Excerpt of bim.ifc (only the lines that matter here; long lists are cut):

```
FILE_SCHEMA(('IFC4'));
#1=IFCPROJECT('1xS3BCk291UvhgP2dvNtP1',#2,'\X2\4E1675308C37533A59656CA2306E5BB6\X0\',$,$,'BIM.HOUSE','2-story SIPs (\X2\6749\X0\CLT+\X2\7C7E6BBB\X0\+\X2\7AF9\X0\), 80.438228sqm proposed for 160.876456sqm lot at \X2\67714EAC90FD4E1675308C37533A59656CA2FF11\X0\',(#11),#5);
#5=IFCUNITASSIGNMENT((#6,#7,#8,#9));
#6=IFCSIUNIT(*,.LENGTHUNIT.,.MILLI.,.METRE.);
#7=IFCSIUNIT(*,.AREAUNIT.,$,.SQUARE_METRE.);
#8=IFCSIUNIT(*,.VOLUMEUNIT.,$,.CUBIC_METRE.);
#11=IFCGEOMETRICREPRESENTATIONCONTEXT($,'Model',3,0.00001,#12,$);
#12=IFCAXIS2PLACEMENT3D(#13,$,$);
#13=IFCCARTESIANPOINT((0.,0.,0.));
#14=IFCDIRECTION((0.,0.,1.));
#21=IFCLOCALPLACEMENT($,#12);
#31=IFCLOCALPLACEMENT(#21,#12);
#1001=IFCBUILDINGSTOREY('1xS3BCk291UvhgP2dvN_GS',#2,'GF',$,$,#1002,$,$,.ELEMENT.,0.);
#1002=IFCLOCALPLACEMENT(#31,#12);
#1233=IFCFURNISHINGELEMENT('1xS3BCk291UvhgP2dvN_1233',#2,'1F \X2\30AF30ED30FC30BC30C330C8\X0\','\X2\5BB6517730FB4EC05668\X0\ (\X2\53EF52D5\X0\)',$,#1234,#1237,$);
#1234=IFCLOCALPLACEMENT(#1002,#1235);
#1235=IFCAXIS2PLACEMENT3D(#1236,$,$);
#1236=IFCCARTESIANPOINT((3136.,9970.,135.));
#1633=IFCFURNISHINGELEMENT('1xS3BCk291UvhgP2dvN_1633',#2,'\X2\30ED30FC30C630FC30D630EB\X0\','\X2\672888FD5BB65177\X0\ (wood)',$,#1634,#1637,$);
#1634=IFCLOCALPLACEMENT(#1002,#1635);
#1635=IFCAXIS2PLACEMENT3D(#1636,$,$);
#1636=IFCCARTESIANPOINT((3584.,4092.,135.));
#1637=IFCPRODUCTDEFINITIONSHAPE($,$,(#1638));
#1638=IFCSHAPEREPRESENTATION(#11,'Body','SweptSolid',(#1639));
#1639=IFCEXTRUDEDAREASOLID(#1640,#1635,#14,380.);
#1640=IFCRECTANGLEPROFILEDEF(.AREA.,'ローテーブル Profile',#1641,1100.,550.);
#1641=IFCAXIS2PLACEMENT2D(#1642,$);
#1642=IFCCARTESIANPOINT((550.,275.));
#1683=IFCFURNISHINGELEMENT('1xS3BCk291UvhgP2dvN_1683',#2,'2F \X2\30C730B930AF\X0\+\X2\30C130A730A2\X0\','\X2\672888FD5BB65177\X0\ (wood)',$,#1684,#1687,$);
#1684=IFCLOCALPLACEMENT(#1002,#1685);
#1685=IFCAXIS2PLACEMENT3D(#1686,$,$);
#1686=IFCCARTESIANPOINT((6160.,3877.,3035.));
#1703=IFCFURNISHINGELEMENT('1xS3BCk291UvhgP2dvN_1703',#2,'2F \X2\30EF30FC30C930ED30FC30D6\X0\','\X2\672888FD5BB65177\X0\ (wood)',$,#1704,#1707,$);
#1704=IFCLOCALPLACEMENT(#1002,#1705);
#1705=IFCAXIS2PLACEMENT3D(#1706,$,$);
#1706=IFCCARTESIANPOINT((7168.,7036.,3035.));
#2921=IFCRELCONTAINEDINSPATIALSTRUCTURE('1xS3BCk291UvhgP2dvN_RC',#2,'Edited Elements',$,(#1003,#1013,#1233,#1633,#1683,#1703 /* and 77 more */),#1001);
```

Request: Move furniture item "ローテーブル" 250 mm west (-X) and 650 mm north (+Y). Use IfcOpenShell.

```python
import ifcopenshell
import ifcopenshell.api.geometry
import ifcopenshell.util.placement
import ifcopenshell.util.unit

model = ifcopenshell.open("bim.ifc")
unit_scale = ifcopenshell.util.unit.calculate_unit_scale(model)

item = model.by_id(1633)
matrix = ifcopenshell.util.placement.get_local_placement(item.ObjectPlacement)
matrix[0, 3] -= 0.25 / unit_scale
matrix[1, 3] += 0.65 / unit_scale
ifcopenshell.api.geometry.edit_object_placement(model, product=item, matrix=matrix, is_si=False)

print(ifcopenshell.util.placement.get_local_placement(item.ObjectPlacement).round(3) + 0.0)

model.write("bim_v2.ifc")
```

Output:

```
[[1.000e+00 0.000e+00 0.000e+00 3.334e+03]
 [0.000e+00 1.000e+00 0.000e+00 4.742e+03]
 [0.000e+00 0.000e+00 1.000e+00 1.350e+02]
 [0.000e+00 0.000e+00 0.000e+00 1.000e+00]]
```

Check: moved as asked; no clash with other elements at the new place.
